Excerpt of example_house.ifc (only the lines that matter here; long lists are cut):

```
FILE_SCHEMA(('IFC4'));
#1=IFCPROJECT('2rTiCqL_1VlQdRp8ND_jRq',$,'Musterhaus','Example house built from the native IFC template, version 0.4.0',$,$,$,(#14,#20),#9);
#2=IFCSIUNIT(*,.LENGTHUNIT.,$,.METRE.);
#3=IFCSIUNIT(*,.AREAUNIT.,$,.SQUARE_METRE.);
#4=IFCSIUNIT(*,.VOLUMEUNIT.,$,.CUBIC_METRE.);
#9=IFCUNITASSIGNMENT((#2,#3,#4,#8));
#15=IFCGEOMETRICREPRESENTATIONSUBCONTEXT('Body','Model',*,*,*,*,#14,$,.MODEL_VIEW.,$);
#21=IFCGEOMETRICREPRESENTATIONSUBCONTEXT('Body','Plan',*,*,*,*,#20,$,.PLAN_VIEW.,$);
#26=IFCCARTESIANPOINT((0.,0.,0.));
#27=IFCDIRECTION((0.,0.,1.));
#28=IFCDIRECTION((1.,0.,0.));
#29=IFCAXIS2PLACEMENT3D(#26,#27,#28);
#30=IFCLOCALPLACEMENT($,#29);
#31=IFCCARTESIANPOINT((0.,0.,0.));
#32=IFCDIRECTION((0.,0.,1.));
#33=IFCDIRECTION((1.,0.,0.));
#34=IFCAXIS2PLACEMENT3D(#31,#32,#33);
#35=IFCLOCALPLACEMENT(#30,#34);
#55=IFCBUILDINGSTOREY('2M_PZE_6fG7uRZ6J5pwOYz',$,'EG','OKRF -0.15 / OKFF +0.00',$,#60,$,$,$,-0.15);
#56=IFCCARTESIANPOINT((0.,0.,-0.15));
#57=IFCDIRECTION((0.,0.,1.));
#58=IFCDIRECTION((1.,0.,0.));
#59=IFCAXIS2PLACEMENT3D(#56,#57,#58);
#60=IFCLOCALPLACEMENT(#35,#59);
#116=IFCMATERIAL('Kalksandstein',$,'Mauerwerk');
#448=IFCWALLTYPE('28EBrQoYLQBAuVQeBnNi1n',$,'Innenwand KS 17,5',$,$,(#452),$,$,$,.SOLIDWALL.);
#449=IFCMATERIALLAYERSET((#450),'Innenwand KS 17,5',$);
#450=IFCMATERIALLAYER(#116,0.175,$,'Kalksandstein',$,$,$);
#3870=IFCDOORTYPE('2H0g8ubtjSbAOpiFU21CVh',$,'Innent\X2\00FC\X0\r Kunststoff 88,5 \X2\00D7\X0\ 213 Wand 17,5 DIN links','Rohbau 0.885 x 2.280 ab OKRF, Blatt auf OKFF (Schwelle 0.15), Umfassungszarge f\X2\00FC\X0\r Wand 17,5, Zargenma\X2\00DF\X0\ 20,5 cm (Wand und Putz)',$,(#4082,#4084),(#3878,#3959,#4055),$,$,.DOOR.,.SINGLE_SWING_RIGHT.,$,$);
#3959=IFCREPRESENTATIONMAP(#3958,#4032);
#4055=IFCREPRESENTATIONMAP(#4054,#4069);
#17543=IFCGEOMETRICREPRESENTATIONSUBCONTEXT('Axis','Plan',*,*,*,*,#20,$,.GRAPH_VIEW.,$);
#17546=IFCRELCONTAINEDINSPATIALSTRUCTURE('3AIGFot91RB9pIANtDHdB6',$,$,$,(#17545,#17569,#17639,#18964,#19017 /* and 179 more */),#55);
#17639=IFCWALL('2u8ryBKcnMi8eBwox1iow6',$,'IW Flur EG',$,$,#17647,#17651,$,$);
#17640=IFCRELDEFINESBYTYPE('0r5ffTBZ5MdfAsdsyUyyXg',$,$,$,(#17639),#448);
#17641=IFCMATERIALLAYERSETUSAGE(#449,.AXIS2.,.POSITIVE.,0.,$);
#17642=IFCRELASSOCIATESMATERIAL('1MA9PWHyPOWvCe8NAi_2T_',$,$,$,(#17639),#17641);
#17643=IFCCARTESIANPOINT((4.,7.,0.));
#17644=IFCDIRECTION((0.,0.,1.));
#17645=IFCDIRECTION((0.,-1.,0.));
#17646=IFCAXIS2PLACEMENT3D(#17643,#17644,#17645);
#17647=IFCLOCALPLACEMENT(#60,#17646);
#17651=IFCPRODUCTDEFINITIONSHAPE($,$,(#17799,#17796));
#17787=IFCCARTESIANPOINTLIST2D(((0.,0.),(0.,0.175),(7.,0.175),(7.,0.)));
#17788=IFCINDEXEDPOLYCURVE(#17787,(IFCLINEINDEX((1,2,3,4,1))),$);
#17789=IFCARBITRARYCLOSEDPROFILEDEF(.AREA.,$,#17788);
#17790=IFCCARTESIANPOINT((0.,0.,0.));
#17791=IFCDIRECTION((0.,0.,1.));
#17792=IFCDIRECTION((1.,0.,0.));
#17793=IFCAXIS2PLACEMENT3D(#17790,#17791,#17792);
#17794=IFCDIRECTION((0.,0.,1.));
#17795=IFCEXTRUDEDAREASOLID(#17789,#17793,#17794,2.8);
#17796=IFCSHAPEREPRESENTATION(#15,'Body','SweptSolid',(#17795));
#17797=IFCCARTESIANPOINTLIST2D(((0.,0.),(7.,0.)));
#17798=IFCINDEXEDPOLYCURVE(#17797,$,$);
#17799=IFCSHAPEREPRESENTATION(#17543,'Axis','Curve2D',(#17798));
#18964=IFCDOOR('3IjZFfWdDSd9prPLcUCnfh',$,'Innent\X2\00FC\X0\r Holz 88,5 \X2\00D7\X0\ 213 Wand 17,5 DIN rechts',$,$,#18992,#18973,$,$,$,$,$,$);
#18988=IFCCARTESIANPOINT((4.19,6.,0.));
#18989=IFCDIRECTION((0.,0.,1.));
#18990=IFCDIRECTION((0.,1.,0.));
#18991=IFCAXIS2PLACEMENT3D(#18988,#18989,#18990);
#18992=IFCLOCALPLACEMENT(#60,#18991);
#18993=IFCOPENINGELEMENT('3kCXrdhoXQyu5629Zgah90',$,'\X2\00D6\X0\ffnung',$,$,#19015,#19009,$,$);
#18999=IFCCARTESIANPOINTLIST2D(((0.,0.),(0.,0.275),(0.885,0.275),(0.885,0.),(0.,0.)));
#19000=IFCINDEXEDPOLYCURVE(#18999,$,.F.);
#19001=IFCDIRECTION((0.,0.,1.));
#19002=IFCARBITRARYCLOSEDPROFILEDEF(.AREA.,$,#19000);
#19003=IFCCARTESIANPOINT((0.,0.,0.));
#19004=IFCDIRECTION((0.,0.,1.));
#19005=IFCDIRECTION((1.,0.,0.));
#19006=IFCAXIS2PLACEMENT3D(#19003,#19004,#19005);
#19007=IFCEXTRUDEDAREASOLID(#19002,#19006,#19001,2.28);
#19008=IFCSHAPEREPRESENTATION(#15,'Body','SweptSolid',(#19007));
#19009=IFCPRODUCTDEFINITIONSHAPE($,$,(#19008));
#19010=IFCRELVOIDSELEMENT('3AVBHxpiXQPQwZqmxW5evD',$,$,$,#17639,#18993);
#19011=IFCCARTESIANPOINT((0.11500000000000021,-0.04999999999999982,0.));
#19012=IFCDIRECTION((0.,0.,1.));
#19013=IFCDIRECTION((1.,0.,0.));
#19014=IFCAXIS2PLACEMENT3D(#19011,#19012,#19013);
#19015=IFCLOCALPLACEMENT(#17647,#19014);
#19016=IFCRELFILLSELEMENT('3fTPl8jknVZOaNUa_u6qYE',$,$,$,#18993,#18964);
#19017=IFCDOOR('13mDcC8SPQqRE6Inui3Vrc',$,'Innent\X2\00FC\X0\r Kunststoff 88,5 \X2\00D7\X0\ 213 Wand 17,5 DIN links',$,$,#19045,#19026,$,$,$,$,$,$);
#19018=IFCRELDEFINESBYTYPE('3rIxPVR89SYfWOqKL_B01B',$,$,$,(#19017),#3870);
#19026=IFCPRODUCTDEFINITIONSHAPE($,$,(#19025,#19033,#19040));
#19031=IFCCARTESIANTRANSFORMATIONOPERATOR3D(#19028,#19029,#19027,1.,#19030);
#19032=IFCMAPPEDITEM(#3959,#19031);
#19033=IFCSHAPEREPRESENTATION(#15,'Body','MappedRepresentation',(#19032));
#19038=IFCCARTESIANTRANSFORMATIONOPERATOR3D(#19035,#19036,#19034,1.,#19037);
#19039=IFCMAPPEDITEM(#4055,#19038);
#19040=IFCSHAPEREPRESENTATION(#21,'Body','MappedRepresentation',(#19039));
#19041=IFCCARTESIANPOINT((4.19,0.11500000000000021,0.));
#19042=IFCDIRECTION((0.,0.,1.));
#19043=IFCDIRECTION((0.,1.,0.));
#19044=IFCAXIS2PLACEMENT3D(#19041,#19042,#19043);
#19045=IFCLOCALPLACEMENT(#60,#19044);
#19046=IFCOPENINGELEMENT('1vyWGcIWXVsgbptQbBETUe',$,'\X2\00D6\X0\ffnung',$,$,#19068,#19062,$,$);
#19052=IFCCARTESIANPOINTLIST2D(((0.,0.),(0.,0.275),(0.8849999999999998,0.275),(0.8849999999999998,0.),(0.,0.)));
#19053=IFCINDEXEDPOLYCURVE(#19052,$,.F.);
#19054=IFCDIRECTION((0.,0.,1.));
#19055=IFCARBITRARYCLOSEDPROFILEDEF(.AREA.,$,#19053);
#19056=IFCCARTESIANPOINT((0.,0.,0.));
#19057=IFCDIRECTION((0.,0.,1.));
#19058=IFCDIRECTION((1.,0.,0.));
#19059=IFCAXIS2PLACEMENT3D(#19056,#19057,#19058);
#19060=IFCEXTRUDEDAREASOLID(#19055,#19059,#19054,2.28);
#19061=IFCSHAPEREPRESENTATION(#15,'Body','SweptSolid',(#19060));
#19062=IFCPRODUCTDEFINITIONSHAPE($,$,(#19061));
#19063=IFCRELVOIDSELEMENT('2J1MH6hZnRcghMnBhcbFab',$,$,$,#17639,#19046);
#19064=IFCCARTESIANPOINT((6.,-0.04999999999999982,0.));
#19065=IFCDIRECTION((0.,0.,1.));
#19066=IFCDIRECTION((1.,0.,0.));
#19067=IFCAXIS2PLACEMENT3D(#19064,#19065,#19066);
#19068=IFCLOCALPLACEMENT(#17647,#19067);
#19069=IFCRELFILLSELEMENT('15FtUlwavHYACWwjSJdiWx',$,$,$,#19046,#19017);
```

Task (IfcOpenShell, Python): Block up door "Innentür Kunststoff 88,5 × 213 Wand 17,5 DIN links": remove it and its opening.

```python
import ifcopenshell
import ifcopenshell.api.feature
import ifcopenshell.api.root
import ifcopenshell.geom
import ifcopenshell.util.shape

model = ifcopenshell.open("example_house.ifc")
settings = ifcopenshell.geom.settings()


def volume(element):
    """Net volume in cubic metres, openings subtracted."""
    shape = ifcopenshell.geom.create_shape(settings, element)
    return ifcopenshell.util.shape.get_volume(shape.geometry)


door = model.by_id(19017)
opening = door.FillsVoids[0].RelatingOpeningElement
wall = opening.VoidsElements[0].RelatingBuildingElement
before = volume(wall)

ifcopenshell.api.root.remove_product(model, product=door)
ifcopenshell.api.feature.remove_feature(model, feature=opening)

after = volume(wall)

print(f"wall volume {before:.3f} -> {after:.3f} m3")

model.write("example_house_edited.ifc")
```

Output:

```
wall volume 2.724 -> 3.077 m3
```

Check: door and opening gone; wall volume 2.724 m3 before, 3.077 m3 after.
